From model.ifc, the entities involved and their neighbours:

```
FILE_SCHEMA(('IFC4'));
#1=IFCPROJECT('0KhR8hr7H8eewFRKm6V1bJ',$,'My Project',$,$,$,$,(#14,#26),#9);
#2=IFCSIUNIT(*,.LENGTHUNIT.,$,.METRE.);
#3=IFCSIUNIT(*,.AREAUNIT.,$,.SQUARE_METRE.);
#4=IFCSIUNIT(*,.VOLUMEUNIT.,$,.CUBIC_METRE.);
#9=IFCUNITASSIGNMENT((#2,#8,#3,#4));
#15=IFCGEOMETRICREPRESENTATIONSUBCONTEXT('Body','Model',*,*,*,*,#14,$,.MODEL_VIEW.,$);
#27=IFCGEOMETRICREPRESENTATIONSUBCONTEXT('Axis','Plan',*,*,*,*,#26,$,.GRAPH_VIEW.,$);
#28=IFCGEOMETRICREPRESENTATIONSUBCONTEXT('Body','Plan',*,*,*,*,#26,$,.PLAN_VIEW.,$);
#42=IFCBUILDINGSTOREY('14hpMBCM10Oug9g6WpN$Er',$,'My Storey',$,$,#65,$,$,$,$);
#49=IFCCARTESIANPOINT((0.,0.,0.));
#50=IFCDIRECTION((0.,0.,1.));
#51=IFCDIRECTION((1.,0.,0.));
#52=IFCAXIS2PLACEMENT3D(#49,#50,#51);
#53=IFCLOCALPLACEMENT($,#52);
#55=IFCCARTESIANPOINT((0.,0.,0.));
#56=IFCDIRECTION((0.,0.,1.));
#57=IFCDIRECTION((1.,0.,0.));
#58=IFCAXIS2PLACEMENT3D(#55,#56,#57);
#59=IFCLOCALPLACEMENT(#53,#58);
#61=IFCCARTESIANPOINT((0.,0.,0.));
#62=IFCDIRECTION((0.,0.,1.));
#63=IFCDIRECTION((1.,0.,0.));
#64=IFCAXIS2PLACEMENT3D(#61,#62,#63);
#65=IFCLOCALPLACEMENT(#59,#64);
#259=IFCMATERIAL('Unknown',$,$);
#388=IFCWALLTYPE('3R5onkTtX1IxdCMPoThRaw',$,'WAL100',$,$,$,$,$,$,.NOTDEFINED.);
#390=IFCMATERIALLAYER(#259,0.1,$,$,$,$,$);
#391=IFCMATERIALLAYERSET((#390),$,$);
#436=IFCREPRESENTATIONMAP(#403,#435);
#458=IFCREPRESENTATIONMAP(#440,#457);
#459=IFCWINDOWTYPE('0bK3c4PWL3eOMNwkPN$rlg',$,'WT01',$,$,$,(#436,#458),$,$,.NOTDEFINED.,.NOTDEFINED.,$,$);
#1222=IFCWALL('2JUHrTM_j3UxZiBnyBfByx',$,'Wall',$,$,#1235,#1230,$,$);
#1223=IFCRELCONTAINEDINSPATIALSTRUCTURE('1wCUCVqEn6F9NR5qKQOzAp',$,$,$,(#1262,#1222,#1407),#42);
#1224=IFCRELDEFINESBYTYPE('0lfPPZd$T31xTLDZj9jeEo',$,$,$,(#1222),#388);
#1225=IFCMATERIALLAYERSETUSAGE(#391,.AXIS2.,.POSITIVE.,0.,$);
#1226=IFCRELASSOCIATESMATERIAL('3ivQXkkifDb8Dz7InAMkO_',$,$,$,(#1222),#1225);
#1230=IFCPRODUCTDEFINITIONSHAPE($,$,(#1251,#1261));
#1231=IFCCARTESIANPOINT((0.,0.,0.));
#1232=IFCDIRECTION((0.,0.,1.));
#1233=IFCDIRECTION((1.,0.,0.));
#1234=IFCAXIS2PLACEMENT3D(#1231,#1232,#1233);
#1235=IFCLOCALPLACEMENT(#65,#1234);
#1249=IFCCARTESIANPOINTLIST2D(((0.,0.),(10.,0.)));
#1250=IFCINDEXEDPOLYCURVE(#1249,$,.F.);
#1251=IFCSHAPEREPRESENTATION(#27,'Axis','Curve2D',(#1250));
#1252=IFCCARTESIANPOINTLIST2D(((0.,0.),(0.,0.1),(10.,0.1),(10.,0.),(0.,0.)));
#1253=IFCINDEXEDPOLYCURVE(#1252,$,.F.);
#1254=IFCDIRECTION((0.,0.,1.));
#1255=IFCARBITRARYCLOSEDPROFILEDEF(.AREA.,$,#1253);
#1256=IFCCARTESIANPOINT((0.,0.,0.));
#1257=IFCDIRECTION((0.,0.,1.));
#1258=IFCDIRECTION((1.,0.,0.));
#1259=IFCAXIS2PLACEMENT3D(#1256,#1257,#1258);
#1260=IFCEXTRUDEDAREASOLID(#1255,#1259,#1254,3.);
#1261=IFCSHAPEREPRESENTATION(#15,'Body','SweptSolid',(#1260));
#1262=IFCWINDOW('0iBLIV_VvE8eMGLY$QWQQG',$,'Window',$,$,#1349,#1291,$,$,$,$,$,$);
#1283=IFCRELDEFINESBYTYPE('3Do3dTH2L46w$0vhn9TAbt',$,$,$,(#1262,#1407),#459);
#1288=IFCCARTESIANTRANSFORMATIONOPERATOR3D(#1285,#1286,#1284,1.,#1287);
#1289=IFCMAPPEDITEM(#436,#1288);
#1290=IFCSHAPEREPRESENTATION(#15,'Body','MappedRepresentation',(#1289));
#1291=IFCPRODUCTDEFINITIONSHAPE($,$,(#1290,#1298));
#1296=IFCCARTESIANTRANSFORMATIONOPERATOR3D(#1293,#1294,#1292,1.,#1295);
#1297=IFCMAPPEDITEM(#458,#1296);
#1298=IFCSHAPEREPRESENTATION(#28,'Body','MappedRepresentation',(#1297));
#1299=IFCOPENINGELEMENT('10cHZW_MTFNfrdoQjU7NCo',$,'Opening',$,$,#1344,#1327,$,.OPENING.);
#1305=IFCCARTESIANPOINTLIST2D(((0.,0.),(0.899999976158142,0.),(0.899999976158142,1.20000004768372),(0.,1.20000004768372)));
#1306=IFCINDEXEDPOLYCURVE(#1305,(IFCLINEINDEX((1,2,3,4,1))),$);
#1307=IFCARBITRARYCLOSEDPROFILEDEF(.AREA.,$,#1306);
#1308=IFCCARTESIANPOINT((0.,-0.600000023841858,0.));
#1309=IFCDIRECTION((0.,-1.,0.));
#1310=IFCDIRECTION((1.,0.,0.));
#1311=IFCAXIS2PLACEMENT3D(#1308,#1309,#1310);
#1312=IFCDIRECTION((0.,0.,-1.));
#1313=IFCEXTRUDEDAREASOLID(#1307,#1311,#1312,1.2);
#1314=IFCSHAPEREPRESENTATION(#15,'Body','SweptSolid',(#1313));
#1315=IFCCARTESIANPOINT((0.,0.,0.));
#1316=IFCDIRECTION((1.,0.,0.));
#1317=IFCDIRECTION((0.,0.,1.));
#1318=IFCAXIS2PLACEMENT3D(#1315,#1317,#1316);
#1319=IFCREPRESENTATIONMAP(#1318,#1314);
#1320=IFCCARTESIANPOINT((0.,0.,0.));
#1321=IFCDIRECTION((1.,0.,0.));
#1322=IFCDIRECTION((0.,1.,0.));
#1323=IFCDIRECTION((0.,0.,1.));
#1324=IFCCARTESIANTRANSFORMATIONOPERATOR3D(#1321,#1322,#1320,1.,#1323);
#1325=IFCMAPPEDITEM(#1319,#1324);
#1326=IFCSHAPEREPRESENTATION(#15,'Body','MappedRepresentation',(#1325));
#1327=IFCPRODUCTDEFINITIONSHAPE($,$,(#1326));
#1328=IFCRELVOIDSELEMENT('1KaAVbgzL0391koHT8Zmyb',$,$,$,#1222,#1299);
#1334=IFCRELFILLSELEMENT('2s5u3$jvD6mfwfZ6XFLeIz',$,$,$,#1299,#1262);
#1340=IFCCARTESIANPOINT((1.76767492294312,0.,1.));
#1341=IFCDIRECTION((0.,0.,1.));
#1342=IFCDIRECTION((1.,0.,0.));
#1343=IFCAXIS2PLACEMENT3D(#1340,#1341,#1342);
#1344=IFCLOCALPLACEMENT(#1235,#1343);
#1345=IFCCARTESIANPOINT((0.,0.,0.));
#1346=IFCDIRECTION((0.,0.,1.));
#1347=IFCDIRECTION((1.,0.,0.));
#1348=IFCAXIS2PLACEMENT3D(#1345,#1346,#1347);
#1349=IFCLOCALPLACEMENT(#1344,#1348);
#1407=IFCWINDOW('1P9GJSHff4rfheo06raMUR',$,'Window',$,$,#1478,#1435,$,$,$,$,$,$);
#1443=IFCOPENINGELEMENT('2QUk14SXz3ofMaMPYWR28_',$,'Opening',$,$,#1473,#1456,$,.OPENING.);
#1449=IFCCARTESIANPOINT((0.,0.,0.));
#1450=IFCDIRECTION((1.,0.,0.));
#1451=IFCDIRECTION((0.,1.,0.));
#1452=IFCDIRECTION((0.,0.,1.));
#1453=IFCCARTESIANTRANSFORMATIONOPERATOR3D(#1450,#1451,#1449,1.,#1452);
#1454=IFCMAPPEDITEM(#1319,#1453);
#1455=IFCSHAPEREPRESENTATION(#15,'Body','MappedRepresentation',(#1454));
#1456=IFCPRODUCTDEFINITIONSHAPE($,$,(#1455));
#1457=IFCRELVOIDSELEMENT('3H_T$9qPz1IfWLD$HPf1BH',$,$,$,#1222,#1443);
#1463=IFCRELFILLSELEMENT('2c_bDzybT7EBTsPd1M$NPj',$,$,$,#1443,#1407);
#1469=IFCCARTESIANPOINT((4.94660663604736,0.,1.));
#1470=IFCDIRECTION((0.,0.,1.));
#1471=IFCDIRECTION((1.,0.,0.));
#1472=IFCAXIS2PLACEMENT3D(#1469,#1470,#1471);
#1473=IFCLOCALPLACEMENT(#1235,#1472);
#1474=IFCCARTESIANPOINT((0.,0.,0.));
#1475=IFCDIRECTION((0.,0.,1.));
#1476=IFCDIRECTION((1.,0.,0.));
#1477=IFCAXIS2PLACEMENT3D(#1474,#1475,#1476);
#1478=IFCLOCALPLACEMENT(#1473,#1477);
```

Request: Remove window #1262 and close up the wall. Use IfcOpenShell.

```python
import ifcopenshell
import ifcopenshell.api.feature
import ifcopenshell.api.root
import ifcopenshell.geom
import ifcopenshell.util.shape

model = ifcopenshell.open("model.ifc")
settings = ifcopenshell.geom.settings()


def volume(element):
    """Net volume in cubic metres, openings subtracted."""
    shape = ifcopenshell.geom.create_shape(settings, element)
    return ifcopenshell.util.shape.get_volume(shape.geometry)


window = model.by_guid("0iBLIV_VvE8eMGLY$QWQQG")
opening = window.FillsVoids[0].RelatingOpeningElement
wall = opening.VoidsElements[0].RelatingBuildingElement
before = volume(wall)

ifcopenshell.api.root.remove_product(model, product=window)
ifcopenshell.api.feature.remove_feature(model, feature=opening)

after = volume(wall)

print(f"wall volume {before:.3f} -> {after:.3f} m3")

model.write("model-out.ifc")
```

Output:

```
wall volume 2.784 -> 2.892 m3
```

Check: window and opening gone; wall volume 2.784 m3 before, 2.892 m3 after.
